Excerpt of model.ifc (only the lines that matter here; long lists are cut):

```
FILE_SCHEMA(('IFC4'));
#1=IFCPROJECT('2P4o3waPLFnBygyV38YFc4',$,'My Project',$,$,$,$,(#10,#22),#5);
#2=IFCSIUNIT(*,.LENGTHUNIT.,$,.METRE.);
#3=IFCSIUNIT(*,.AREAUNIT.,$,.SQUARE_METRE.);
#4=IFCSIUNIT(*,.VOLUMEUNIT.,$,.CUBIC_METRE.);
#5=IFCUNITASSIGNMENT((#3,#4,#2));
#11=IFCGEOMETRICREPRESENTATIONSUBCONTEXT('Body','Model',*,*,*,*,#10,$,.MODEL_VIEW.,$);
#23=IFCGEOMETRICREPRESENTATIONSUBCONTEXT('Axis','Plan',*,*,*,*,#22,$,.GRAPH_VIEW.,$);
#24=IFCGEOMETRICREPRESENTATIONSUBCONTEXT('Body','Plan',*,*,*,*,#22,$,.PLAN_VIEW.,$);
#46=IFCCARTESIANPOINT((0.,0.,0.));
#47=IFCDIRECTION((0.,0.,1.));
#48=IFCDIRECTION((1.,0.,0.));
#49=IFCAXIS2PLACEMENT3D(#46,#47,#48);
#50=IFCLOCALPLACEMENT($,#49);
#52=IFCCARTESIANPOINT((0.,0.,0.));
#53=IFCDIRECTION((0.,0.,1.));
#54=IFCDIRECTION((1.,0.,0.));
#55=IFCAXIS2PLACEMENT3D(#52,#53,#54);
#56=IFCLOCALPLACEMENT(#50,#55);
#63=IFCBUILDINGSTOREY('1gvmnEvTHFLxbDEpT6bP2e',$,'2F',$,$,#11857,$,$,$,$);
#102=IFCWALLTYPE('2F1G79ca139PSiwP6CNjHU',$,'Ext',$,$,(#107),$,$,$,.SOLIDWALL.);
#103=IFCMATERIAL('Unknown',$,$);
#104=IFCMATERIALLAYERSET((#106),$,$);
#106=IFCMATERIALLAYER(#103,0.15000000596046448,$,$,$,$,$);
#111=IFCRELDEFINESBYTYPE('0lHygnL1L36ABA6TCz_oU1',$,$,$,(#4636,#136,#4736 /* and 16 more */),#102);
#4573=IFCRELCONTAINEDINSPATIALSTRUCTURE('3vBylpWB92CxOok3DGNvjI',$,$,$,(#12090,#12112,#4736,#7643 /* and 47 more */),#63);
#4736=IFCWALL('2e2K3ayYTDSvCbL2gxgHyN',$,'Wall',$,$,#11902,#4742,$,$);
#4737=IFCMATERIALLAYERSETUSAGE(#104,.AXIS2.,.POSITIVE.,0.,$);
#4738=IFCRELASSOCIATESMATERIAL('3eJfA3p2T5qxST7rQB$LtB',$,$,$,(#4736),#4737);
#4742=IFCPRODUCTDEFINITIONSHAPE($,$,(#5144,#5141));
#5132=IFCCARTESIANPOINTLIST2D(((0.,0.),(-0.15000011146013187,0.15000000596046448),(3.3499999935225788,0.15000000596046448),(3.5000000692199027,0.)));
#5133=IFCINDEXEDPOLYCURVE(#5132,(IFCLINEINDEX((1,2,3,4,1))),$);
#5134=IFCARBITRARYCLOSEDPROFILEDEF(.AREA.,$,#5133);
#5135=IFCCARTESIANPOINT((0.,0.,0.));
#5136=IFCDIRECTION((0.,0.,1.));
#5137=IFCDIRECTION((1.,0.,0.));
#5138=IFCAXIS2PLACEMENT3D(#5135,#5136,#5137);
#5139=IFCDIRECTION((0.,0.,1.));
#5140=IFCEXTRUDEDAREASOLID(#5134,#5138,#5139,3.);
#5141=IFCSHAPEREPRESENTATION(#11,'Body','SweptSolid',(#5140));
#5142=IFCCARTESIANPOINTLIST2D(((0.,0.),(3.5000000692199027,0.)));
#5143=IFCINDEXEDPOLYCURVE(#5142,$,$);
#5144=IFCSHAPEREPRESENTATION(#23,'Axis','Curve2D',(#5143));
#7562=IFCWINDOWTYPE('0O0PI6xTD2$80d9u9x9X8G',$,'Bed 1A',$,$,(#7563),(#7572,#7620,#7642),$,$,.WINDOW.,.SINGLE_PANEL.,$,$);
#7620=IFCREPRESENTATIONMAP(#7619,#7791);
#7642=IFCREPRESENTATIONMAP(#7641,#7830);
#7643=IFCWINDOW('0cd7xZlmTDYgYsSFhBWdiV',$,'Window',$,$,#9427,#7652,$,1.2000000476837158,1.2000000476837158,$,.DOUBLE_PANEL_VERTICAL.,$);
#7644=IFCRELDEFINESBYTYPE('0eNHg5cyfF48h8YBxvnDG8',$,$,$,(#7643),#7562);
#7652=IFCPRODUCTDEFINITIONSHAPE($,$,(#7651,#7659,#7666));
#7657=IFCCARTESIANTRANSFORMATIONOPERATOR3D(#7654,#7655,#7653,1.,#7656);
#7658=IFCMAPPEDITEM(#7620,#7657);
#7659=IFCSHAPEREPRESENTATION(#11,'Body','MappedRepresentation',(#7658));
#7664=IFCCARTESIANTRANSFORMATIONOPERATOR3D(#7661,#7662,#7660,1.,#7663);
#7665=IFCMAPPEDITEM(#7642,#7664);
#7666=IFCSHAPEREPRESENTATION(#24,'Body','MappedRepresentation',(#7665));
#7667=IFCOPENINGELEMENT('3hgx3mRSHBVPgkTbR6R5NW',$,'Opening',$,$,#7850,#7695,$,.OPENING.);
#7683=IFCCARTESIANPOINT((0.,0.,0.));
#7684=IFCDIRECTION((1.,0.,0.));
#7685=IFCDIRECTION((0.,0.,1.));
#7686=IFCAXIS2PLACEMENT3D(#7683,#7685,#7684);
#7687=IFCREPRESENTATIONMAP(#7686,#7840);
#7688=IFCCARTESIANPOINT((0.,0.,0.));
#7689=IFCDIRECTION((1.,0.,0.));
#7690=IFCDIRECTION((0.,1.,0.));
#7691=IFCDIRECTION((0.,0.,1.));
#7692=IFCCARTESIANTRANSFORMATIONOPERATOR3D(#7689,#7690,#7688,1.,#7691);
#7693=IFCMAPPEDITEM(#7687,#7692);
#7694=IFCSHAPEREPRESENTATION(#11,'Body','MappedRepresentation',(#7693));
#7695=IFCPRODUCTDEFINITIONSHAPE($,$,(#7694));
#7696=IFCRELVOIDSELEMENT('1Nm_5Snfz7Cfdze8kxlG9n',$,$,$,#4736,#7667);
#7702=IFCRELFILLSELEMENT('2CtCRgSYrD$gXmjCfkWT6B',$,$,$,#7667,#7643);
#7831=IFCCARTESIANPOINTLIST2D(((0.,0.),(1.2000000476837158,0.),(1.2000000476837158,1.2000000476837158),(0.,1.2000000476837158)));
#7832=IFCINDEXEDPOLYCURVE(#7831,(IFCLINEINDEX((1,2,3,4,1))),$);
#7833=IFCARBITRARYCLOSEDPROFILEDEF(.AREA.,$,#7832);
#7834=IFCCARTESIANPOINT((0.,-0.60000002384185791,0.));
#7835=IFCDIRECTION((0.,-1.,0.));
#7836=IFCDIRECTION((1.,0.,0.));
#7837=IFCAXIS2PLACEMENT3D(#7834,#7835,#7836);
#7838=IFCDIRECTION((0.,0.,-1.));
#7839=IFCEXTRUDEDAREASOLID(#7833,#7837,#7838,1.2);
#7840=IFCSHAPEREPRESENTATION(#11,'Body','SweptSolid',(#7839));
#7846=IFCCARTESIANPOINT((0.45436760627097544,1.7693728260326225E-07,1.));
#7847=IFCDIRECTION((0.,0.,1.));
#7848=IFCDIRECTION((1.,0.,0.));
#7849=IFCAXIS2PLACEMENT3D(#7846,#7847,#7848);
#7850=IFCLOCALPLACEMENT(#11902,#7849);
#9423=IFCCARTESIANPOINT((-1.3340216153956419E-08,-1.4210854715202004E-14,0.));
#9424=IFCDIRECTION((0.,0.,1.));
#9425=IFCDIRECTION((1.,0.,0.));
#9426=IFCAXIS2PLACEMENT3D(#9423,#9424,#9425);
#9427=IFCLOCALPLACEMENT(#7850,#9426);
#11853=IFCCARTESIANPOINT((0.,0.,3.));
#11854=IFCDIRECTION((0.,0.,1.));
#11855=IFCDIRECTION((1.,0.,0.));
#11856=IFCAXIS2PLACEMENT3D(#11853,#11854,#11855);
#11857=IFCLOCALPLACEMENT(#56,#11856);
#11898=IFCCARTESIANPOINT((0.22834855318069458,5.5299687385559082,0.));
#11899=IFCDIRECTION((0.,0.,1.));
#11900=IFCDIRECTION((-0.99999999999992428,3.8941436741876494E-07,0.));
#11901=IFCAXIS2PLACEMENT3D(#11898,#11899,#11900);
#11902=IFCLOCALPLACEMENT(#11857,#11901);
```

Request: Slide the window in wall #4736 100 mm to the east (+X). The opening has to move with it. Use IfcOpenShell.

```python
import ifcopenshell
import ifcopenshell.api.geometry
import ifcopenshell.util.placement
import ifcopenshell.util.unit

model = ifcopenshell.open("model.ifc")
unit_scale = ifcopenshell.util.unit.calculate_unit_scale(model)

window = model.by_guid("0cd7xZlmTDYgYsSFhBWdiV")
opening = window.FillsVoids[0].RelatingOpeningElement
wall = opening.VoidsElements[0].RelatingBuildingElement

wall_matrix = ifcopenshell.util.placement.get_local_placement(wall.ObjectPlacement)
shift = wall_matrix[:3, 0] * -0.1 / unit_scale
before = ifcopenshell.util.placement.get_local_placement(window.ObjectPlacement)[:3, 3].copy()

# The window is placed relative to its opening, so it follows when the opening moves.
matrix = ifcopenshell.util.placement.get_local_placement(opening.ObjectPlacement)
matrix[:3, 3] += shift
ifcopenshell.api.geometry.edit_object_placement(
    model, product=opening, matrix=matrix, is_si=False, should_transform_children=True
)

after = ifcopenshell.util.placement.get_local_placement(window.ObjectPlacement)[:3, 3]
print("window moved by", (after - before).round(3) + 0.0)

model.write("model_updated.ifc")
```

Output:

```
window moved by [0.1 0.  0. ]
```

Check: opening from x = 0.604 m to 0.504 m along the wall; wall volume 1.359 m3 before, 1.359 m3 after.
